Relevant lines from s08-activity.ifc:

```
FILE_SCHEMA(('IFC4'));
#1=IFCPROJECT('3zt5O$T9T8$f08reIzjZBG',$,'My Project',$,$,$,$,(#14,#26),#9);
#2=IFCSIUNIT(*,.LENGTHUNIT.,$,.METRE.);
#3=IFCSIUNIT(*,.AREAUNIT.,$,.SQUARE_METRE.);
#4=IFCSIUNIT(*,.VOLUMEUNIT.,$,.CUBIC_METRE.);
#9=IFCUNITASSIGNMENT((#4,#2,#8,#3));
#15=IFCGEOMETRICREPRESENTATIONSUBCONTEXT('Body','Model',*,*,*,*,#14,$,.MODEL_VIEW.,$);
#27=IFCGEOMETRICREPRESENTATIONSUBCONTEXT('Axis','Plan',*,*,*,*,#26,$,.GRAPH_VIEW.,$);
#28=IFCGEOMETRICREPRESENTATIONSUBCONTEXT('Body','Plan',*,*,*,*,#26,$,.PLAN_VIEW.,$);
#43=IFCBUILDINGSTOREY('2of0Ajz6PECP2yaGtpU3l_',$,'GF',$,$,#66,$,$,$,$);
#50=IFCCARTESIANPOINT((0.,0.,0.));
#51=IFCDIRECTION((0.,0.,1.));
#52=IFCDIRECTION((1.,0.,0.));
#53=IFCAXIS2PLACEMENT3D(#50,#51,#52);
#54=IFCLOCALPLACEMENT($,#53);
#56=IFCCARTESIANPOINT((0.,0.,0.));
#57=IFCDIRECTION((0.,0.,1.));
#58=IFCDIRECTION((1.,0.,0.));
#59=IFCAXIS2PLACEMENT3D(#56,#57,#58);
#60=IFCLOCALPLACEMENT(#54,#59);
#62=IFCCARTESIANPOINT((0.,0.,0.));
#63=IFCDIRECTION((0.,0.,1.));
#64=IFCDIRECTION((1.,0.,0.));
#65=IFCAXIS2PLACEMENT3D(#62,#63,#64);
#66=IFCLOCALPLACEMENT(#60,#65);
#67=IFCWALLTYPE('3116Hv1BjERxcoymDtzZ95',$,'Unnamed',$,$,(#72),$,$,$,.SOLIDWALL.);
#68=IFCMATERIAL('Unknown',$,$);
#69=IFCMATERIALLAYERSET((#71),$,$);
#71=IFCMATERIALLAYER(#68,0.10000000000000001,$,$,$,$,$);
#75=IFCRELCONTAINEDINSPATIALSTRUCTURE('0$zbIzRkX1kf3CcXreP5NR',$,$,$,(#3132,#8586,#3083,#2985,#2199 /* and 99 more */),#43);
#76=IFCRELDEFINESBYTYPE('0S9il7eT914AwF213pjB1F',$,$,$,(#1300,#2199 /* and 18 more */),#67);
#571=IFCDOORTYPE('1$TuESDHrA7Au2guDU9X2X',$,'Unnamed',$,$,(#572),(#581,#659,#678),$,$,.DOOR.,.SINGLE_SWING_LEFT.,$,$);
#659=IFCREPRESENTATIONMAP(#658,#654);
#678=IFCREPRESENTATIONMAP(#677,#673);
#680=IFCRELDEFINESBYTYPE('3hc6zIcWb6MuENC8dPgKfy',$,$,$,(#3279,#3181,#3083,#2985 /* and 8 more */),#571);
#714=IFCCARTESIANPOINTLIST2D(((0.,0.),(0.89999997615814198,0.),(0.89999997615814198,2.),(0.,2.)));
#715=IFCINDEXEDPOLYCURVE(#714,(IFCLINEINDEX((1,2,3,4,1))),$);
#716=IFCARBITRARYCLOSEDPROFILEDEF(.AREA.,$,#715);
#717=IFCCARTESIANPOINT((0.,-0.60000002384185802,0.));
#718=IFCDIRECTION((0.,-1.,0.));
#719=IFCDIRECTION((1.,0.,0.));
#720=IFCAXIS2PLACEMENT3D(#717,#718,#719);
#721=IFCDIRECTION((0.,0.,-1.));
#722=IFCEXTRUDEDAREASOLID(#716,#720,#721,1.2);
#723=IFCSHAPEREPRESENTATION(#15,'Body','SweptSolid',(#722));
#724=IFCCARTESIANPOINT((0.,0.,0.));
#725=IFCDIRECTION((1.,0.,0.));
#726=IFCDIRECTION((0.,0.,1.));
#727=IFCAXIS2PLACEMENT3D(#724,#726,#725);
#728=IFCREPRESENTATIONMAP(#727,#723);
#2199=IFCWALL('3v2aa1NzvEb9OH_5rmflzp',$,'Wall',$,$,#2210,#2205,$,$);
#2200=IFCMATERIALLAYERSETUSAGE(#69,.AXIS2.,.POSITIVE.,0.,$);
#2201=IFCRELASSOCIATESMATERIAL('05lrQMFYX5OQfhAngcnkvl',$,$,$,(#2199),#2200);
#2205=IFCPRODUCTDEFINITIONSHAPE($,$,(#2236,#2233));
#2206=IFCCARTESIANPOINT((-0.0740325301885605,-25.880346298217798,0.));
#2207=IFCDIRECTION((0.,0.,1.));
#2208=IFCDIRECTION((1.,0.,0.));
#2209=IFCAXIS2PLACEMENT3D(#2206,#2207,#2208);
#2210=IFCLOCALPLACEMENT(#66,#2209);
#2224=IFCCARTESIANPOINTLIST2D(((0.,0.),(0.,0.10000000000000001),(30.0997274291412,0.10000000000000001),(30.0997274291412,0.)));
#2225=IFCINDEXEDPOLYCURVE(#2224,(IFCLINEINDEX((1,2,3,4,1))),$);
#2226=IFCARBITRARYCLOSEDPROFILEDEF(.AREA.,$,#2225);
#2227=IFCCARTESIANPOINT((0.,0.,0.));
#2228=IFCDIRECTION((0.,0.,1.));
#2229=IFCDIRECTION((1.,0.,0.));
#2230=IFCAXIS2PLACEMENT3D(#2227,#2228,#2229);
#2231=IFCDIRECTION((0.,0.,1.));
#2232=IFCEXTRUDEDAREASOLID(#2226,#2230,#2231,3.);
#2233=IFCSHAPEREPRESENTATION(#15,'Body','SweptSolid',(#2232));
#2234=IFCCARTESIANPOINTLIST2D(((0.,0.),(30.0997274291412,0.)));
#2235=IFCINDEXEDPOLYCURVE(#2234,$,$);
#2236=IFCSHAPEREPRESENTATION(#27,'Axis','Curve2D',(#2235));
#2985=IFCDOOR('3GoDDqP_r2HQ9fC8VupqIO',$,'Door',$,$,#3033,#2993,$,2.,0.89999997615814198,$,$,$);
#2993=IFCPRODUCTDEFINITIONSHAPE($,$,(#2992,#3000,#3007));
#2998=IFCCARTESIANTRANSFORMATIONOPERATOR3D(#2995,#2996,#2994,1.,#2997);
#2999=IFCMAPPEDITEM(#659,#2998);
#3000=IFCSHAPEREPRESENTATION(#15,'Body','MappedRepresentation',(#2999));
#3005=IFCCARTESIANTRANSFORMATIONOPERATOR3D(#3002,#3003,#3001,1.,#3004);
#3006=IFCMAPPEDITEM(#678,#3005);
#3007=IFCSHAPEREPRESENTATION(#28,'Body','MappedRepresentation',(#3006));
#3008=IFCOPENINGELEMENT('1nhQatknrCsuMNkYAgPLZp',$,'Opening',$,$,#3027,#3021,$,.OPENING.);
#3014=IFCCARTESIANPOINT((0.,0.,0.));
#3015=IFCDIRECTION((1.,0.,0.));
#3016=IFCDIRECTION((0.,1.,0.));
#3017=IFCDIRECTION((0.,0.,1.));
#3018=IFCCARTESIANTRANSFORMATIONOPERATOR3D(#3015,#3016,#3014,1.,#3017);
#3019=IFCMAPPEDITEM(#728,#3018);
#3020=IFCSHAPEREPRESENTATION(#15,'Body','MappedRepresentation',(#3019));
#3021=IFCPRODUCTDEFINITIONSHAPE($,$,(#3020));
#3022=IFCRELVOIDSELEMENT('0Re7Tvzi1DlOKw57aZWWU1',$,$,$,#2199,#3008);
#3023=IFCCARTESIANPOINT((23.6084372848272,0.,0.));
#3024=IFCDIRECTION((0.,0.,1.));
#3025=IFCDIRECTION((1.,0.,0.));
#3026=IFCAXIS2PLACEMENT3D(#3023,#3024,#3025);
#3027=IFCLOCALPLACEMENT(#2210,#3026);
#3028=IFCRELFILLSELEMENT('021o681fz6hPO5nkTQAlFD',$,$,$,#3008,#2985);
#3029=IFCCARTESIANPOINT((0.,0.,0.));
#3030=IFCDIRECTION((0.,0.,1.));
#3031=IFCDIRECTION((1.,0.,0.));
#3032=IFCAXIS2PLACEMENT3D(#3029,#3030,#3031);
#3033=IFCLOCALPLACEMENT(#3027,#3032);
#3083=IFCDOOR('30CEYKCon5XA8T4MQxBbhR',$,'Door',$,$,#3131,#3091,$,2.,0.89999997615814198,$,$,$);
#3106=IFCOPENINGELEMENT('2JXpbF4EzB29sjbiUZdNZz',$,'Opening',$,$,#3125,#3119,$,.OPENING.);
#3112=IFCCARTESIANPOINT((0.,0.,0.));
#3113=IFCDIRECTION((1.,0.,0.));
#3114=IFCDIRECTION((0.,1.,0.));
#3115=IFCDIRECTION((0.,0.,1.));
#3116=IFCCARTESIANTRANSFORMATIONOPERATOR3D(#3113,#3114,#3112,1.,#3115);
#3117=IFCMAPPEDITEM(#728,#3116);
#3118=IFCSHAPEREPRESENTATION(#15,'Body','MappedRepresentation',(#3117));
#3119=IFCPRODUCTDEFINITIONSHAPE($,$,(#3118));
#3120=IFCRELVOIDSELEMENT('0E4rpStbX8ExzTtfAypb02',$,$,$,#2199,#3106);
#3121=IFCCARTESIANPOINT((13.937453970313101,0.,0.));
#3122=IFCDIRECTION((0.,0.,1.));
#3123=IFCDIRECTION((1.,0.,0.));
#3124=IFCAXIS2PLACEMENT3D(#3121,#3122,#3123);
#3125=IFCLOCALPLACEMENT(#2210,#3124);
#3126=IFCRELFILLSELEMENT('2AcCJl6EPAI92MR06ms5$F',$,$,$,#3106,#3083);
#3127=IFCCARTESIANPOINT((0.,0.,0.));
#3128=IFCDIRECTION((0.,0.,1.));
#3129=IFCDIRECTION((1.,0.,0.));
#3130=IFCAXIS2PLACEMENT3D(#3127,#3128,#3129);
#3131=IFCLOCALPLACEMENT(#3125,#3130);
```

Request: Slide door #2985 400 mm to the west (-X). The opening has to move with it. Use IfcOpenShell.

```python
import ifcopenshell
import ifcopenshell.api.geometry
import ifcopenshell.util.placement
import ifcopenshell.util.unit

model = ifcopenshell.open("s08-activity.ifc")
unit_scale = ifcopenshell.util.unit.calculate_unit_scale(model)

door = model.by_guid("3GoDDqP_r2HQ9fC8VupqIO")
opening = door.FillsVoids[0].RelatingOpeningElement
wall = opening.VoidsElements[0].RelatingBuildingElement

wall_matrix = ifcopenshell.util.placement.get_local_placement(wall.ObjectPlacement)
shift = wall_matrix[:3, 0] * -0.4 / unit_scale
before = ifcopenshell.util.placement.get_local_placement(door.ObjectPlacement)[:3, 3].copy()

# The door is placed relative to its opening, so it follows when the opening moves.
matrix = ifcopenshell.util.placement.get_local_placement(opening.ObjectPlacement)
matrix[:3, 3] += shift
ifcopenshell.api.geometry.edit_object_placement(
    model, product=opening, matrix=matrix, is_si=False, should_transform_children=True
)

after = ifcopenshell.util.placement.get_local_placement(door.ObjectPlacement)[:3, 3]
print("door moved by", (after - before).round(3) + 0.0)

model.write("s08-activity_rev.ifc")
```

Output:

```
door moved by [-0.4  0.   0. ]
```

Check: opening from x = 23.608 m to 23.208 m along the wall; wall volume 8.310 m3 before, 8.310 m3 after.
